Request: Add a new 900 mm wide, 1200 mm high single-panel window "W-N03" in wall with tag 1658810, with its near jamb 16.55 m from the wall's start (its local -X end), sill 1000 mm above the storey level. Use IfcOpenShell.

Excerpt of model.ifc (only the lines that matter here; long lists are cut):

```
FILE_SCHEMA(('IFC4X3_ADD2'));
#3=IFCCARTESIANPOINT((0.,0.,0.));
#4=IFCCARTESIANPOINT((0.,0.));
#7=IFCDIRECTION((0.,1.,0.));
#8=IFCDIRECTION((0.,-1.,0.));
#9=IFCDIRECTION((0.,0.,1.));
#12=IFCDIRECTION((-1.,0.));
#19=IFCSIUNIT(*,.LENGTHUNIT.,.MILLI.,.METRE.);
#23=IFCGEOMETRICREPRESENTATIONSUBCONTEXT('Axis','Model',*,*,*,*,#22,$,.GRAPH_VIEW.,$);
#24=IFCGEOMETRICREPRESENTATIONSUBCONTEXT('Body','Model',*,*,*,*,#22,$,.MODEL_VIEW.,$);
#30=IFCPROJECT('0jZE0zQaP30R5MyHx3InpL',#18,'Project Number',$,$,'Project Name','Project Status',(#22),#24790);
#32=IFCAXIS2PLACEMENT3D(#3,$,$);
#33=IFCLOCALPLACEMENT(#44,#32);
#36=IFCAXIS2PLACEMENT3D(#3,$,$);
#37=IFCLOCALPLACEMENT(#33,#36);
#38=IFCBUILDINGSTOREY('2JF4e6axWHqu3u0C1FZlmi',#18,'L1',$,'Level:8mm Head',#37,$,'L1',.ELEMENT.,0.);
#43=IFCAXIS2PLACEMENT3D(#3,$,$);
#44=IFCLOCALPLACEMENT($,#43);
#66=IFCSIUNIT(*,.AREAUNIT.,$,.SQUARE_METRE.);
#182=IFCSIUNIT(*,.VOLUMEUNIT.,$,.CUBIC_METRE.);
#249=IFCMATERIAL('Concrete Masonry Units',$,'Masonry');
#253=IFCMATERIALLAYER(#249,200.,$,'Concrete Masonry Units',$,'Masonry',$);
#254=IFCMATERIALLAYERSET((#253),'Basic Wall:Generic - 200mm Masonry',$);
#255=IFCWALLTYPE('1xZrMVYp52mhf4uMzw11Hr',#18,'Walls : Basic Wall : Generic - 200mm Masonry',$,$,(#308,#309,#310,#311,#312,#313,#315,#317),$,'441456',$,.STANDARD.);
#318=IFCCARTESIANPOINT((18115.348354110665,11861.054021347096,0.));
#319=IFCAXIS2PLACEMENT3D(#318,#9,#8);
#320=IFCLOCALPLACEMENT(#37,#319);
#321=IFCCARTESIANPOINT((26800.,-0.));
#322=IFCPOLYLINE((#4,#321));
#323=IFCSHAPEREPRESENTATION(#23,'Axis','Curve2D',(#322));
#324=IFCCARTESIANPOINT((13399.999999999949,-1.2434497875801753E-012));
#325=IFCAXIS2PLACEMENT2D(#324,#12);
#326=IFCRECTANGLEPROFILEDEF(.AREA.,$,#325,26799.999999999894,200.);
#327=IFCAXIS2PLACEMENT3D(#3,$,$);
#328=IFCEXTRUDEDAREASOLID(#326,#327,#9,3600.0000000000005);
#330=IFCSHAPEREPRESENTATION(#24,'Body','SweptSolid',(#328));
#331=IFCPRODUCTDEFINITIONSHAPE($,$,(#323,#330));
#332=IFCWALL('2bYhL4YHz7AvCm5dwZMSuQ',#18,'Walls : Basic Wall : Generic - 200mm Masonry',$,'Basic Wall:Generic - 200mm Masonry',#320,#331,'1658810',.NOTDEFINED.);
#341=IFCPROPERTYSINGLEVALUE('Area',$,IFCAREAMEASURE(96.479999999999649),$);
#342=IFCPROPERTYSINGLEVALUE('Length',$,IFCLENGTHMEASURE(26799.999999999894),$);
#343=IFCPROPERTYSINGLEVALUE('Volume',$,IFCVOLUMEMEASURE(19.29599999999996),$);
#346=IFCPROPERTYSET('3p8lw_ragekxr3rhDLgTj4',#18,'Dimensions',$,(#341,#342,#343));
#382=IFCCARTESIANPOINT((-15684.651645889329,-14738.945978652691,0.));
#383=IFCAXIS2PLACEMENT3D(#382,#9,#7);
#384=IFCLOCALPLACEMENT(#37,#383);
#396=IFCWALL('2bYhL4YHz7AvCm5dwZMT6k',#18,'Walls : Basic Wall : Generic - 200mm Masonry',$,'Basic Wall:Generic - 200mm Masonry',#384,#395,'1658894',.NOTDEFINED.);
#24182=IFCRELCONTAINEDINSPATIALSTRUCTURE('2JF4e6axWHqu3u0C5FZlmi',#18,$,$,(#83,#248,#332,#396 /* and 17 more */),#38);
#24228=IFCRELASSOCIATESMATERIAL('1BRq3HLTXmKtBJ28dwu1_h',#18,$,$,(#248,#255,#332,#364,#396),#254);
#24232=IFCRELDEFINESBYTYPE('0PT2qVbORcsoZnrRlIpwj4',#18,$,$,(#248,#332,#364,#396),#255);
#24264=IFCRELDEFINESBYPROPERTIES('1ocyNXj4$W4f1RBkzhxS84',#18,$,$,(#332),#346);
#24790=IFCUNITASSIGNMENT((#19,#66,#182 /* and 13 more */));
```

```python
import numpy as np
import ifcopenshell
import ifcopenshell.api.feature
import ifcopenshell.api.geometry
import ifcopenshell.api.pset
import ifcopenshell.api.root
import ifcopenshell.api.spatial
import ifcopenshell.geom
import ifcopenshell.util.element
import ifcopenshell.util.placement
import ifcopenshell.util.representation
import ifcopenshell.util.shape
import ifcopenshell.util.unit

model = ifcopenshell.open("model.ifc")
unit_scale = ifcopenshell.util.unit.calculate_unit_scale(model)
area_scale = ifcopenshell.util.unit.calculate_unit_scale(model, "AREAUNIT")
volume_scale = ifcopenshell.util.unit.calculate_unit_scale(model, "VOLUMEUNIT")
settings = ifcopenshell.geom.settings()


def volume(element):
    """Net volume in cubic metres, openings subtracted."""
    shape = ifcopenshell.geom.create_shape(settings, element)
    return ifcopenshell.util.shape.get_volume(shape.geometry)


wall = model.by_guid("2bYhL4YHz7AvCm5dwZMSuQ")
storey = ifcopenshell.util.element.get_container(wall, ifc_class="IfcBuildingStorey")
context = ifcopenshell.util.representation.get_context(model, "Model", "Body", "MODEL_VIEW")
before = volume(wall)

width, height, from_end, sill = 0.9, 1.2, 16.55, 1  # metres

# The wall runs along its own X axis, and the end named is its -X end.
wall_shape = ifcopenshell.geom.create_shape(settings, wall)
x, y, z = ifcopenshell.util.shape.get_vertices(wall_shape.geometry).T
start = x.min() + from_end
face, thickness = float(y.min()), float(y.max() - y.min())
wall_matrix = ifcopenshell.util.placement.get_local_placement(wall.ObjectPlacement)
level = ifcopenshell.util.placement.get_local_placement(storey.ObjectPlacement)[2, 3]


def in_wall(x, y):
    """Placement at x, y metres in the wall's axes, at sill height."""
    matrix = wall_matrix.copy()
    matrix[:, 3] = wall_matrix @ np.array([x / unit_scale, y / unit_scale, 0.0, 1.0])
    matrix[2, 3] = level + sill / unit_scale
    return matrix


# Opening: a box that overshoots both wall faces by 50 mm.
opening = ifcopenshell.api.root.create_entity(model, ifc_class="IfcOpeningElement", predefined_type="OPENING")
box = ifcopenshell.api.geometry.add_wall_representation(
    model, context=context, length=width, height=height, thickness=thickness + 0.1
)
ifcopenshell.api.geometry.assign_representation(model, product=opening, representation=box)
ifcopenshell.api.geometry.edit_object_placement(model, product=opening, matrix=in_wall(start, face - 0.05), is_si=False)
ifcopenshell.api.feature.add_feature(model, feature=opening, element=wall)

window = ifcopenshell.api.root.create_entity(model, ifc_class="IfcWindow", name="W-N03", predefined_type="WINDOW")
window.OverallWidth, window.OverallHeight = width / unit_scale, height / unit_scale
window.PartitioningType = "SINGLE_PANEL"
body = ifcopenshell.api.geometry.add_window_representation(
    model,
    context=context,
    overall_width=window.OverallWidth,
    overall_height=window.OverallHeight,
    partition_type="SINGLE_PANEL",
)
ifcopenshell.api.geometry.assign_representation(model, product=window, representation=body)
ifcopenshell.api.spatial.assign_container(model, products=[window], relating_structure=storey)
ifcopenshell.api.feature.add_filling(model, opening=opening, element=window)

# Centre the window in the wall's thickness.
ifcopenshell.api.geometry.edit_object_placement(model, product=window, matrix=in_wall(start, face), is_si=False)
window_shape = ifcopenshell.geom.create_shape(settings, window)
depth = ifcopenshell.util.shape.get_vertices(window_shape.geometry)[:, 1]
offset = face + thickness / 2 - (depth.min() + depth.max()) / 2
ifcopenshell.api.geometry.edit_object_placement(model, product=window, matrix=in_wall(start, offset), is_si=False)

after = volume(wall)

# Update the wall's stored quantities.
pset = model.by_id(ifcopenshell.util.element.get_pset(wall, "Dimensions", should_inherit=False)["id"])
ifcopenshell.api.pset.edit_pset(model, pset=pset, properties={
    "Area": model.create_entity("IfcAreaMeasure", after / thickness / area_scale),
    "Volume": model.create_entity("IfcVolumeMeasure", after / volume_scale),
})

print(f"wall volume {before:.3f} -> {after:.3f} m3")

model.write("model-out.ifc")
```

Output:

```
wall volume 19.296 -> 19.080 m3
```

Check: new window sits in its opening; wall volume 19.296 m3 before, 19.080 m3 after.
